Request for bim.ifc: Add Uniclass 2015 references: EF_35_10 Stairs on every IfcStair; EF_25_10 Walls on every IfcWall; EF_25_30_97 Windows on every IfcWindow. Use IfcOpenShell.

First a look at what the model holds.

```python
import ifcopenshell

model = ifcopenshell.open("bim.ifc")
print(model.schema)
print("classifications:", [c.Name for c in model.by_type("IfcClassification")])
for ifc_class in ("IfcDoor", "IfcRoof", "IfcStair", "IfcWall", "IfcWindow"):
    print(ifc_class, len(model.by_type(ifc_class)))
```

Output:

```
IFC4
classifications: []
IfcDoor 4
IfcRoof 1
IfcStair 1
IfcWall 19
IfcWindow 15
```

```python
import ifcopenshell
import ifcopenshell.api.classification

model = ifcopenshell.open("bim.ifc")

system = ifcopenshell.api.classification.add_classification(model, classification="Uniclass 2015")

codes = {
    "IfcStair": ("EF_35_10", "Stairs"),
    "IfcWall": ("EF_25_10", "Walls"),
    "IfcWindow": ("EF_25_30_97", "Windows"),
}
for ifc_class, (code, name) in codes.items():
    products = model.by_type(ifc_class)
    ifcopenshell.api.classification.add_reference(
        model, products=products, classification=system, identification=code, name=name
    )
    print(code, len(products))

model.write("bim_v2.ifc")
```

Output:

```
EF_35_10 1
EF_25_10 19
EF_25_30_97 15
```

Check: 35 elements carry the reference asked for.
